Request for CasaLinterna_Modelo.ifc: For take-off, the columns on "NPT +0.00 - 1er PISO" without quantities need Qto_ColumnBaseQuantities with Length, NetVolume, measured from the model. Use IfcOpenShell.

First a look at what the model holds.

```python
import ifcopenshell
import ifcopenshell.util.element
import ifcopenshell.util.unit

model = ifcopenshell.open("CasaLinterna_Modelo.ifc")
print(model.schema)
for unit_type in ("LENGTHUNIT", "AREAUNIT", "VOLUMEUNIT"):
    print(unit_type, ifcopenshell.util.unit.calculate_unit_scale(model, unit_type))
storey = next(s for s in model.by_type("IfcBuildingStorey") if s.Name == "NPT +0.00 - 1er PISO")
columns = [e for e in ifcopenshell.util.element.get_decomposition(storey) if e.is_a("IfcColumn")]
for e in sorted(columns, key=lambda e: e.id()):
    print(e.id(), e.is_a(), e.Name, list(ifcopenshell.util.element.get_psets(e, qtos_only=True)), sep=" | ")
```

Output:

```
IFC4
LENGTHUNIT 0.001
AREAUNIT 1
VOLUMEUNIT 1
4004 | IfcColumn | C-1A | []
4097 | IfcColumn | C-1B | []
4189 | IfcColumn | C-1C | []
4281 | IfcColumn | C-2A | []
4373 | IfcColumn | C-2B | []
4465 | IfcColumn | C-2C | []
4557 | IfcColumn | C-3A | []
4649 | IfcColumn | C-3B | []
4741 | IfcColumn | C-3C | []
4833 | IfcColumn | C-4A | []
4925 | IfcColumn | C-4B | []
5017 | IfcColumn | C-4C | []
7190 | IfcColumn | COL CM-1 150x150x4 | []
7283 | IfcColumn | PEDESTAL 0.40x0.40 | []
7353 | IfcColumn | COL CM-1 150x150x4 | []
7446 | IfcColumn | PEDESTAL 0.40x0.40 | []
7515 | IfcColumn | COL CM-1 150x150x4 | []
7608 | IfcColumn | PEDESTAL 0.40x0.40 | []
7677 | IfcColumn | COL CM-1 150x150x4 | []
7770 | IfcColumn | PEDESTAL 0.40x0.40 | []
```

```python
import ifcopenshell
import ifcopenshell.api.pset
import ifcopenshell.geom
import ifcopenshell.util.element
import ifcopenshell.util.shape
import ifcopenshell.util.unit

model = ifcopenshell.open("CasaLinterna_Modelo.ifc")
unit_scale = ifcopenshell.util.unit.calculate_unit_scale(model)
volume_scale = ifcopenshell.util.unit.calculate_unit_scale(model, "VOLUMEUNIT")
settings = ifcopenshell.geom.settings()

storey = next(s for s in model.by_type("IfcBuildingStorey") if s.Name == "NPT +0.00 - 1er PISO")
columns = [e for e in ifcopenshell.util.element.get_decomposition(storey) if e.is_a("IfcColumn")]

for e in sorted(columns, key=lambda e: e.id()):
    if ifcopenshell.util.element.get_psets(e, qtos_only=True, should_inherit=False):
        continue
    # Geometry comes back in metres, in the element's own axes.
    shape = ifcopenshell.geom.create_shape(settings, e)
    values = {
        "Length": ifcopenshell.util.shape.get_z(shape.geometry) / unit_scale,
        "NetVolume": ifcopenshell.util.shape.get_volume(shape.geometry) / volume_scale,
    }
    qto = ifcopenshell.api.pset.add_qto(model, product=e, name="Qto_ColumnBaseQuantities")
    ifcopenshell.api.pset.edit_qto(model, qto=qto, properties=values)
    print(e.id(), {k: round(v, 3) for k, v in values.items()})

model.write("CasaLinterna_Modelo_v2.ifc")
```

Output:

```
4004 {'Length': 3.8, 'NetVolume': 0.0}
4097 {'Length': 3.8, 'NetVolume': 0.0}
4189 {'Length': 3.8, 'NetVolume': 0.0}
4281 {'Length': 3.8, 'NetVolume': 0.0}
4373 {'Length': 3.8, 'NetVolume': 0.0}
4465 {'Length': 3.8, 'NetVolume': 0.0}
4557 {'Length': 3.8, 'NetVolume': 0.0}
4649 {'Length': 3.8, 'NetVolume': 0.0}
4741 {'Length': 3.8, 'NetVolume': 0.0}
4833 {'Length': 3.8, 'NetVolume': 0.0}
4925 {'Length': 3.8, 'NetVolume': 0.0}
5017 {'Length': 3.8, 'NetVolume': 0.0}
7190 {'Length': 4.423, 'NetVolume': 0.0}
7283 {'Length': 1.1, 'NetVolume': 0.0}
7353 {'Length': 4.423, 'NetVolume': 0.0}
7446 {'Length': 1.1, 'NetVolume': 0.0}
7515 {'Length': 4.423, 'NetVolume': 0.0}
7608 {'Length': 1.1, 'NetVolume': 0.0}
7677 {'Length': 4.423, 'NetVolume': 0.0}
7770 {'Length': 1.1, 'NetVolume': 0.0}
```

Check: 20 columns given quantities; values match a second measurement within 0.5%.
